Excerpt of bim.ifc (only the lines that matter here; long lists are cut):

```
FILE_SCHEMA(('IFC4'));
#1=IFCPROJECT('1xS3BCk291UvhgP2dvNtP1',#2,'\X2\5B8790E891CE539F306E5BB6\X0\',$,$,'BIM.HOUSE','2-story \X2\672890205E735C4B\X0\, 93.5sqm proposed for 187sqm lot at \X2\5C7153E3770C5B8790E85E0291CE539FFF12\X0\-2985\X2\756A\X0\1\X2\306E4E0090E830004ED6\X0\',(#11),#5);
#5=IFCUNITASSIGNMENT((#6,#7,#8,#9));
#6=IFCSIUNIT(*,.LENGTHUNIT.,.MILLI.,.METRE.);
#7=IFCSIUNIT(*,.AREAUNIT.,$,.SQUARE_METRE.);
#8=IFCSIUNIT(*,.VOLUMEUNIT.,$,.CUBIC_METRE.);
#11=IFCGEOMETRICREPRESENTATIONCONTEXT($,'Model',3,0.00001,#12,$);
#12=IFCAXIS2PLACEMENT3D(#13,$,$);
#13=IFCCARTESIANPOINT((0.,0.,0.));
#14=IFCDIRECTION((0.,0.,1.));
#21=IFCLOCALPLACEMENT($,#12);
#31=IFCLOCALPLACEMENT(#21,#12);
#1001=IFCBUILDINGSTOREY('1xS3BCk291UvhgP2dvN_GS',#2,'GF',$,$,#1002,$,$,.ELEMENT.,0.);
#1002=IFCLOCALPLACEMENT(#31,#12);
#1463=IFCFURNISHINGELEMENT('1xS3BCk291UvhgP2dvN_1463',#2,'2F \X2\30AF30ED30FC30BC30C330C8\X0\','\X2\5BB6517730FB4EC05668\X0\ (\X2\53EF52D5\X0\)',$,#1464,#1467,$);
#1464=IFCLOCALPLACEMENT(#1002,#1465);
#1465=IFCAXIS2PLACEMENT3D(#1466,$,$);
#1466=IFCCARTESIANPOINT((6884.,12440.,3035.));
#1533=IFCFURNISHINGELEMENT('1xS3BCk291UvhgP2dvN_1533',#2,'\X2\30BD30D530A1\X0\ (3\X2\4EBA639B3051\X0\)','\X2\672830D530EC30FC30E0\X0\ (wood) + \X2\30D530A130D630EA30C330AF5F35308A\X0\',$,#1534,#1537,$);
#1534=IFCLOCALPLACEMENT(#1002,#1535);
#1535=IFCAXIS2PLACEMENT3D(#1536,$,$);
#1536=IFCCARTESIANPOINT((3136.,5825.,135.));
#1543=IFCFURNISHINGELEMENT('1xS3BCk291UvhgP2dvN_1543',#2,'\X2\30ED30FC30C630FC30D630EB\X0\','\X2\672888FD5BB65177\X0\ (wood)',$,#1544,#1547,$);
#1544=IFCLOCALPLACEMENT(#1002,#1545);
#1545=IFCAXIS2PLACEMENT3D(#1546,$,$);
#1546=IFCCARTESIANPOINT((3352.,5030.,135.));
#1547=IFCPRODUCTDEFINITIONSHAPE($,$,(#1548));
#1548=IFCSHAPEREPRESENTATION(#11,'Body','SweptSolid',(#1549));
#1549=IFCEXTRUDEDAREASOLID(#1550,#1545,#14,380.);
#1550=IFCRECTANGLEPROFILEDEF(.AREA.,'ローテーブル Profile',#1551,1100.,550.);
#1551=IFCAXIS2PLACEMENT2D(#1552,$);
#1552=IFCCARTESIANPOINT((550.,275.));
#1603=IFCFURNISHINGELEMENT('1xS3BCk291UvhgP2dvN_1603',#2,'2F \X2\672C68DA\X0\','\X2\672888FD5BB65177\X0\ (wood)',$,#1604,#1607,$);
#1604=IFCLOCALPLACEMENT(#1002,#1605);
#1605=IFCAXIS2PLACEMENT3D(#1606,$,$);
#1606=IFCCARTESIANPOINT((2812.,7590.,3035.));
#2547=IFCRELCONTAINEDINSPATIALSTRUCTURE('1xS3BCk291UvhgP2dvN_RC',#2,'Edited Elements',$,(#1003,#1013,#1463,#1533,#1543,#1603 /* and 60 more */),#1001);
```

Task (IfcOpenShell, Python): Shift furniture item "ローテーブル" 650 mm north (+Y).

```python
import ifcopenshell
import ifcopenshell.api.geometry
import ifcopenshell.util.placement

model = ifcopenshell.open("bim.ifc")

item = model.by_guid("1xS3BCk291UvhgP2dvN_1543")
matrix = ifcopenshell.util.placement.get_local_placement(item.ObjectPlacement)
matrix[1, 3] += 650.0
ifcopenshell.api.geometry.edit_object_placement(model, product=item, matrix=matrix, is_si=False)

print(ifcopenshell.util.placement.get_local_placement(item.ObjectPlacement).round(3) + 0.0)

model.write("bim-out.ifc")
```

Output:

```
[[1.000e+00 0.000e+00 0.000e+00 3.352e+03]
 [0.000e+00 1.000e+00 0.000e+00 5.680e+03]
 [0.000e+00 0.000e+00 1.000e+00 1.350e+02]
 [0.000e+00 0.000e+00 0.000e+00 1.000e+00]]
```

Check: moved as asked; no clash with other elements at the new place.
